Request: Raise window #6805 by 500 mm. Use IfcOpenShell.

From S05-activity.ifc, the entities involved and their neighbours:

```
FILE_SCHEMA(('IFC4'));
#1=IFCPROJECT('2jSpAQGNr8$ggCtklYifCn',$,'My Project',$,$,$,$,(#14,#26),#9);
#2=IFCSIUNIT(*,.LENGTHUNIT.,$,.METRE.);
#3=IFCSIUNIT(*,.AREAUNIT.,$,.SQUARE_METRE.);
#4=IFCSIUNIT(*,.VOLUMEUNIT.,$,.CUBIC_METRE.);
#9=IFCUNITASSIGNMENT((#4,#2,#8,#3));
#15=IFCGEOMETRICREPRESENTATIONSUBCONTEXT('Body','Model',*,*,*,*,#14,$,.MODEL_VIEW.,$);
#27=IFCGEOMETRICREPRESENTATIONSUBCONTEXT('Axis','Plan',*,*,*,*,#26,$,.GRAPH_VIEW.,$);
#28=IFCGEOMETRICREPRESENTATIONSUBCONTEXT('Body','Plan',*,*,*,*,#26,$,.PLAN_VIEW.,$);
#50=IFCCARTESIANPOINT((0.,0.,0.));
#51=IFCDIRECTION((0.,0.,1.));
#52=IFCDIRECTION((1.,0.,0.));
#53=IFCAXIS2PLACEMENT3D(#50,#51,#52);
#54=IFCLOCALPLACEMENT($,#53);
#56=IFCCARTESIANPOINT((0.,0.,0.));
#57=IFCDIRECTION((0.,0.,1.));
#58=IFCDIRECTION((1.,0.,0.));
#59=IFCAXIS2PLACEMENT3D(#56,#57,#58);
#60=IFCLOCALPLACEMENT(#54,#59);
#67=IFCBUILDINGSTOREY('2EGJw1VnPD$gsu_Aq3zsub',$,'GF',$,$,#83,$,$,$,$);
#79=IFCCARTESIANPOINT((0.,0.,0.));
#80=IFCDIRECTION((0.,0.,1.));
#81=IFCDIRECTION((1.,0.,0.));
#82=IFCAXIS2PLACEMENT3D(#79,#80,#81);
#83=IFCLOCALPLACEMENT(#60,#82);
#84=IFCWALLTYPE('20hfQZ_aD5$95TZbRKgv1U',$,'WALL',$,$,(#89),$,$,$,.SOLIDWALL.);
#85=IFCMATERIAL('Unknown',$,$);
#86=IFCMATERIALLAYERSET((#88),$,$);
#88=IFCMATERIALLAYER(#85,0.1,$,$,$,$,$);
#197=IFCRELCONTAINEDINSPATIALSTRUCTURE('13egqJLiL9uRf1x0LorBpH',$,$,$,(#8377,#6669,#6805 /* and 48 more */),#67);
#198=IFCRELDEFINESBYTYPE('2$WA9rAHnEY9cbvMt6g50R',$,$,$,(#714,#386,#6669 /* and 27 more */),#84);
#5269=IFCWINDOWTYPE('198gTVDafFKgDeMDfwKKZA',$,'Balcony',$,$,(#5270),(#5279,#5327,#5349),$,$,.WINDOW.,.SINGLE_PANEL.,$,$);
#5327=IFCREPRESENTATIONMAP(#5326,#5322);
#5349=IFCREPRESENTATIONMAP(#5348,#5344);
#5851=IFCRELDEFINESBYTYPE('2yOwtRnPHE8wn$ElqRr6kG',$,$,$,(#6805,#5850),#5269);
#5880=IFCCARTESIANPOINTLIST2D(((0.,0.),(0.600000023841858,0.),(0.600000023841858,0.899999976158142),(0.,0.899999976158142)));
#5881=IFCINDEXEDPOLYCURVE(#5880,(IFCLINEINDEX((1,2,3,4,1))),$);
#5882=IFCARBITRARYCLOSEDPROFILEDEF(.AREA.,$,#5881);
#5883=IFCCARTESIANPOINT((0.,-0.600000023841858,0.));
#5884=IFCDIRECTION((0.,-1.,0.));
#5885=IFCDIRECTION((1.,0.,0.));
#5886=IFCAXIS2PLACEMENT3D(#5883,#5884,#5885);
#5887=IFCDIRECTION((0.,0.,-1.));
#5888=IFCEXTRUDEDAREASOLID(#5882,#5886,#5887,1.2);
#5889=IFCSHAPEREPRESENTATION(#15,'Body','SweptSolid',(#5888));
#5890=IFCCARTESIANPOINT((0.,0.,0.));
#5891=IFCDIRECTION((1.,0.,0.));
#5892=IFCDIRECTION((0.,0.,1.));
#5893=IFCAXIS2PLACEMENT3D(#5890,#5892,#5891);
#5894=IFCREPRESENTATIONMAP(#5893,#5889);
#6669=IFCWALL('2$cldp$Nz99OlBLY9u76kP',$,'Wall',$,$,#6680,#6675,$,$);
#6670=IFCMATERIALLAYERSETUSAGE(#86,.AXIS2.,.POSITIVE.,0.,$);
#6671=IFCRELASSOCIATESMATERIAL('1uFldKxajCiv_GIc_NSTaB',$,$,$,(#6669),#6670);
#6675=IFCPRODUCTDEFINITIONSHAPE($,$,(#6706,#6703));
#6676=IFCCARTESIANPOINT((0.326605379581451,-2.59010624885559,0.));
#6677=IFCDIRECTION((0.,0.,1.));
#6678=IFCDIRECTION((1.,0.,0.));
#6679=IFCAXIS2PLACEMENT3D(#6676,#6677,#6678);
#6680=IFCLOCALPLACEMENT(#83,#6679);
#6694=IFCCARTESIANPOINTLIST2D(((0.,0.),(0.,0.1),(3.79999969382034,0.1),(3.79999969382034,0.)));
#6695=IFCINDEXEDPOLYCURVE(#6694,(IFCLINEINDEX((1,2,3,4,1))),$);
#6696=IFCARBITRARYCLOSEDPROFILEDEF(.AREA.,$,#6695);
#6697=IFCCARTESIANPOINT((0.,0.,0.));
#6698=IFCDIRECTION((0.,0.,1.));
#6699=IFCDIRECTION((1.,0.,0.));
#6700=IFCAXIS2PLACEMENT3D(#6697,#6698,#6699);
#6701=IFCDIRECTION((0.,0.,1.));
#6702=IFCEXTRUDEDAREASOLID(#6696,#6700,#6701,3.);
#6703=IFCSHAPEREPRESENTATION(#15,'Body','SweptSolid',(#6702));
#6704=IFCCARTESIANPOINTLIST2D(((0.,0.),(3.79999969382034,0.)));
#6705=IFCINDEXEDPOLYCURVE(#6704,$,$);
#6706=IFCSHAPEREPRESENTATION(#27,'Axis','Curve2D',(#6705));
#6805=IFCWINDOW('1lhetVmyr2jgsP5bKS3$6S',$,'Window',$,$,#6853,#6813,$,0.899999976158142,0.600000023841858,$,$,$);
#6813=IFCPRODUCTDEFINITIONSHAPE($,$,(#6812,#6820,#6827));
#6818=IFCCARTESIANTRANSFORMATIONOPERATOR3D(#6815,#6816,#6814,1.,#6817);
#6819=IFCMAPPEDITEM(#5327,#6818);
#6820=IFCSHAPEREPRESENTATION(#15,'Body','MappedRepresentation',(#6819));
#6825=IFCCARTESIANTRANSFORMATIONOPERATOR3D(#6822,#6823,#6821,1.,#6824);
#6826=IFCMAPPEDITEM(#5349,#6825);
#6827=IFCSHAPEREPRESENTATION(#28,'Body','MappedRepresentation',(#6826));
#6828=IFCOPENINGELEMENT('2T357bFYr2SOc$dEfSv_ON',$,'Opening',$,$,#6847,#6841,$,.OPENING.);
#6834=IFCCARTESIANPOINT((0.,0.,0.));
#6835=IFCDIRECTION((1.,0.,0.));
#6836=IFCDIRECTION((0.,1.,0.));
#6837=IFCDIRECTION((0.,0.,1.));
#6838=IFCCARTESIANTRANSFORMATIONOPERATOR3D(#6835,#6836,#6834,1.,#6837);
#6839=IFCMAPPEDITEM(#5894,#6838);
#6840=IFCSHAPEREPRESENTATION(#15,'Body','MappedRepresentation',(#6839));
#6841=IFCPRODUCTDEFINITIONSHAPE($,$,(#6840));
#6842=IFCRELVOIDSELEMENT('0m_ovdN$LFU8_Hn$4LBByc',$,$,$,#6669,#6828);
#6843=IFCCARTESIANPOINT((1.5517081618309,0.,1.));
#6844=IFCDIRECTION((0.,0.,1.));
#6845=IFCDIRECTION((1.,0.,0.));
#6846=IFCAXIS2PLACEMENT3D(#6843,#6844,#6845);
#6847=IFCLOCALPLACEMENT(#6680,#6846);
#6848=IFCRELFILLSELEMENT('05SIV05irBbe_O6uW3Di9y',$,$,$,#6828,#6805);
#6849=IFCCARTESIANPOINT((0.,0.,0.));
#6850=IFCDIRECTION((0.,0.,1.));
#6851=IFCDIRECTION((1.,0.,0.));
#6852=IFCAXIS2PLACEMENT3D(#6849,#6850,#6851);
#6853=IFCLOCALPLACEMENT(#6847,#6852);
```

```python
import numpy as np
import ifcopenshell
import ifcopenshell.api.geometry
import ifcopenshell.util.placement
import ifcopenshell.util.unit

model = ifcopenshell.open("S05-activity.ifc")
unit_scale = ifcopenshell.util.unit.calculate_unit_scale(model)

window = model.by_guid("1lhetVmyr2jgsP5bKS3$6S")
opening = window.FillsVoids[0].RelatingOpeningElement
dz = 0.5

shift = np.array([0.0, 0.0, dz])
# The window is placed relative to its opening, so it follows when the opening moves.
matrix = ifcopenshell.util.placement.get_local_placement(opening.ObjectPlacement)
matrix[:3, 3] += shift
ifcopenshell.api.geometry.edit_object_placement(
    model, product=opening, matrix=matrix, is_si=False, should_transform_children=True
)

print(f"moved by {dz * unit_scale:+.3f} m")

model.write("S05-activity_updated.ifc")
```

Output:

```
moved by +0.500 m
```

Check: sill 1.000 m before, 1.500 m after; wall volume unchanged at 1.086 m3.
